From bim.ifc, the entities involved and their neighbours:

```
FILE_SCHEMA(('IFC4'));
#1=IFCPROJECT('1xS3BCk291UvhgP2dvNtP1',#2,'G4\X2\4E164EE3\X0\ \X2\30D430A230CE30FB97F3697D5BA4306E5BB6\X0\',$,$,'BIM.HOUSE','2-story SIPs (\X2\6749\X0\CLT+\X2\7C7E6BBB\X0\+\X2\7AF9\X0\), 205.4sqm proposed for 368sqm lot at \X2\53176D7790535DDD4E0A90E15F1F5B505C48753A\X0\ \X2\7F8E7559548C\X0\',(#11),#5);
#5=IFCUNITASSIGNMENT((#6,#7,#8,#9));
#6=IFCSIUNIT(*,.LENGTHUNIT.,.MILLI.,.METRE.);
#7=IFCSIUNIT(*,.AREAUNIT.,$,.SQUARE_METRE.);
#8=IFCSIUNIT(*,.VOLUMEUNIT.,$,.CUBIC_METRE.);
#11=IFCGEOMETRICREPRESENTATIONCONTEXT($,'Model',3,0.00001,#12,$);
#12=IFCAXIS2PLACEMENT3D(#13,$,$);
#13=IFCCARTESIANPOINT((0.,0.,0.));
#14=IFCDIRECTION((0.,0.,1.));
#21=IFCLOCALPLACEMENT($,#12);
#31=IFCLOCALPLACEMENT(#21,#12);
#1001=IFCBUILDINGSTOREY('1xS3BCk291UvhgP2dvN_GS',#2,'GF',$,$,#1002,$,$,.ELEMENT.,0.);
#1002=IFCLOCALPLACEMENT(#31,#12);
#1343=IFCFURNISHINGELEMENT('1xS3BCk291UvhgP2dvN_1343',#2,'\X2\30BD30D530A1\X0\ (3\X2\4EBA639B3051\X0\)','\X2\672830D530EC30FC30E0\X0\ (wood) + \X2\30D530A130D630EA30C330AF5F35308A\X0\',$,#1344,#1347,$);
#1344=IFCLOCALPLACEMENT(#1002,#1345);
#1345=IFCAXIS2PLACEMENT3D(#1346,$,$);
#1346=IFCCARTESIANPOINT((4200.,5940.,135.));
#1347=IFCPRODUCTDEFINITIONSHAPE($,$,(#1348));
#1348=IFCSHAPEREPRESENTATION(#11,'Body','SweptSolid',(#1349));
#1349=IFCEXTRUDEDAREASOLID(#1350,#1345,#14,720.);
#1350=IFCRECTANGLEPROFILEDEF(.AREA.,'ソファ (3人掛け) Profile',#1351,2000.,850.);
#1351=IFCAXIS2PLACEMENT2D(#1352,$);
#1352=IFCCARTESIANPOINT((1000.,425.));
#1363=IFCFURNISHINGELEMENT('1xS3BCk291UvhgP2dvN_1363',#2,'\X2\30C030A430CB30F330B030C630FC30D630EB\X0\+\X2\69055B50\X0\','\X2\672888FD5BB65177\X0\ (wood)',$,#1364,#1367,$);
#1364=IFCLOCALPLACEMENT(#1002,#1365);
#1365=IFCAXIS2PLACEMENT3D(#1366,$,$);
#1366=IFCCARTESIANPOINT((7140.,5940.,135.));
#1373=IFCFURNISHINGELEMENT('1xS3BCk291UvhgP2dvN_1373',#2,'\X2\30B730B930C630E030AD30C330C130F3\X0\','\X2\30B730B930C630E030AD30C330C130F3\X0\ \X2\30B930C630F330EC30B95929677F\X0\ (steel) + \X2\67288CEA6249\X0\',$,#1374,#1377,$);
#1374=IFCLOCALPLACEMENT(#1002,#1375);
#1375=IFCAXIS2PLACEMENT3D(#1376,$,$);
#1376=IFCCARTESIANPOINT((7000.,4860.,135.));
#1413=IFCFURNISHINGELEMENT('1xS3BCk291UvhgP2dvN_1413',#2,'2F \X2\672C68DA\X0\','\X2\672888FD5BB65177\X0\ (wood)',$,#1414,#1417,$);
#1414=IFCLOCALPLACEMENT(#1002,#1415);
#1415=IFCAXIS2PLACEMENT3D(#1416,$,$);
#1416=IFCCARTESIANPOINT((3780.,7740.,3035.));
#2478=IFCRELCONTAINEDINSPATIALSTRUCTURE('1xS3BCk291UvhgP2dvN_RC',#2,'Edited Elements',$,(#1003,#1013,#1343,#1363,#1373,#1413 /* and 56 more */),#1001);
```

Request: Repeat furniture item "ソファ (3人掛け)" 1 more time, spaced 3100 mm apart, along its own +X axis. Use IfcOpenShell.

```python
import ifcopenshell
import ifcopenshell.api.geometry
import ifcopenshell.api.root
import ifcopenshell.util.element
import ifcopenshell.util.placement
import ifcopenshell.util.unit

model = ifcopenshell.open("bim.ifc")
unit_scale = ifcopenshell.util.unit.calculate_unit_scale(model)


def reuse_history(source, copy):
    """copy_class also copies each property set's owner history, people and application; keep the originals."""
    for rel in copy.IsDefinedBy:
        if rel.is_a("IfcRelDefinesByProperties") and (history := rel.RelatingPropertyDefinition.OwnerHistory):
            rel.RelatingPropertyDefinition.OwnerHistory = source.OwnerHistory
            ifcopenshell.util.element.remove_deep2(model, history)


source = model.by_guid("1xS3BCk291UvhgP2dvN_1343")
base = ifcopenshell.util.placement.get_local_placement(source.ObjectPlacement)
step = base[:3, 0] * 3.1 / unit_scale

for i in range(1, 2):
    copy = ifcopenshell.api.root.copy_class(model, product=source)
    copy.Representation = ifcopenshell.util.element.copy_deep(
        model, source.Representation, exclude=["IfcGeometricRepresentationContext", "IfcRepresentationMap"]
    )
    reuse_history(source, copy)
    matrix = base.copy()
    matrix[:3, 3] += i * step
    print("added at", matrix[:3, 3].round(3) + 0.0)
    ifcopenshell.api.geometry.edit_object_placement(model, product=copy, matrix=matrix, is_si=False)

model.write("bim_updated.ifc")
```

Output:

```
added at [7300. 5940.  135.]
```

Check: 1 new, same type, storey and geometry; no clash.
